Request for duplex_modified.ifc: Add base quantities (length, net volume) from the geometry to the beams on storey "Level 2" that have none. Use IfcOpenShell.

First a look at what the model holds.

```python
import ifcopenshell
import ifcopenshell.util.element
import ifcopenshell.util.unit

model = ifcopenshell.open("duplex_modified.ifc")
print(model.schema)
for unit_type in ("LENGTHUNIT", "AREAUNIT", "VOLUMEUNIT"):
    print(unit_type, ifcopenshell.util.unit.calculate_unit_scale(model, unit_type))
storey = next(s for s in model.by_type("IfcBuildingStorey") if s.Name == "Level 2")
beams = [e for e in ifcopenshell.util.element.get_decomposition(storey) if e.is_a("IfcBeam")]
for e in sorted(beams, key=lambda e: e.id()):
    print(e.id(), e.is_a(), e.Name, list(ifcopenshell.util.element.get_psets(e, qtos_only=True)), sep=" | ")
```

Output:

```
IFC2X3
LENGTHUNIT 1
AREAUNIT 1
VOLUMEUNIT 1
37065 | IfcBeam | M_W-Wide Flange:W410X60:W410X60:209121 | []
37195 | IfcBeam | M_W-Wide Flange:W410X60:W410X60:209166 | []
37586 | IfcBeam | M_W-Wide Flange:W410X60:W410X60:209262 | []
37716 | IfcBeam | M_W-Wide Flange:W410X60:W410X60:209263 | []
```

```python
import ifcopenshell
import ifcopenshell.api.pset
import ifcopenshell.geom
import ifcopenshell.util.element
import ifcopenshell.util.shape
import ifcopenshell.util.unit

model = ifcopenshell.open("duplex_modified.ifc")
unit_scale = ifcopenshell.util.unit.calculate_unit_scale(model)
volume_scale = ifcopenshell.util.unit.calculate_unit_scale(model, "VOLUMEUNIT")
settings = ifcopenshell.geom.settings()

storey = next(s for s in model.by_type("IfcBuildingStorey") if s.Name == "Level 2")
beams = [e for e in ifcopenshell.util.element.get_decomposition(storey) if e.is_a("IfcBeam")]

for e in sorted(beams, key=lambda e: e.id()):
    if ifcopenshell.util.element.get_psets(e, qtos_only=True, should_inherit=False):
        continue
    # Geometry comes back in metres, in the element's own axes.
    shape = ifcopenshell.geom.create_shape(settings, e)
    values = {
        "Length": ifcopenshell.util.shape.get_max_xyz(shape.geometry) / unit_scale,
        "NetVolume": ifcopenshell.util.shape.get_volume(shape.geometry) / volume_scale,
    }
    qto = ifcopenshell.api.pset.add_qto(model, product=e, name="BaseQuantities")
    ifcopenshell.api.pset.edit_qto(model, qto=qto, properties=values)
    print(e.id(), {k: round(v, 3) for k, v in values.items()})

model.write("duplex_modified_v2.ifc")
```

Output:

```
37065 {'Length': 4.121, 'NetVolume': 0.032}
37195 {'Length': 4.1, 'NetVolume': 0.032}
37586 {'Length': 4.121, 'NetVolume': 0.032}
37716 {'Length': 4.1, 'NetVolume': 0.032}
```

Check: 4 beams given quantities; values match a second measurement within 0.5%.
